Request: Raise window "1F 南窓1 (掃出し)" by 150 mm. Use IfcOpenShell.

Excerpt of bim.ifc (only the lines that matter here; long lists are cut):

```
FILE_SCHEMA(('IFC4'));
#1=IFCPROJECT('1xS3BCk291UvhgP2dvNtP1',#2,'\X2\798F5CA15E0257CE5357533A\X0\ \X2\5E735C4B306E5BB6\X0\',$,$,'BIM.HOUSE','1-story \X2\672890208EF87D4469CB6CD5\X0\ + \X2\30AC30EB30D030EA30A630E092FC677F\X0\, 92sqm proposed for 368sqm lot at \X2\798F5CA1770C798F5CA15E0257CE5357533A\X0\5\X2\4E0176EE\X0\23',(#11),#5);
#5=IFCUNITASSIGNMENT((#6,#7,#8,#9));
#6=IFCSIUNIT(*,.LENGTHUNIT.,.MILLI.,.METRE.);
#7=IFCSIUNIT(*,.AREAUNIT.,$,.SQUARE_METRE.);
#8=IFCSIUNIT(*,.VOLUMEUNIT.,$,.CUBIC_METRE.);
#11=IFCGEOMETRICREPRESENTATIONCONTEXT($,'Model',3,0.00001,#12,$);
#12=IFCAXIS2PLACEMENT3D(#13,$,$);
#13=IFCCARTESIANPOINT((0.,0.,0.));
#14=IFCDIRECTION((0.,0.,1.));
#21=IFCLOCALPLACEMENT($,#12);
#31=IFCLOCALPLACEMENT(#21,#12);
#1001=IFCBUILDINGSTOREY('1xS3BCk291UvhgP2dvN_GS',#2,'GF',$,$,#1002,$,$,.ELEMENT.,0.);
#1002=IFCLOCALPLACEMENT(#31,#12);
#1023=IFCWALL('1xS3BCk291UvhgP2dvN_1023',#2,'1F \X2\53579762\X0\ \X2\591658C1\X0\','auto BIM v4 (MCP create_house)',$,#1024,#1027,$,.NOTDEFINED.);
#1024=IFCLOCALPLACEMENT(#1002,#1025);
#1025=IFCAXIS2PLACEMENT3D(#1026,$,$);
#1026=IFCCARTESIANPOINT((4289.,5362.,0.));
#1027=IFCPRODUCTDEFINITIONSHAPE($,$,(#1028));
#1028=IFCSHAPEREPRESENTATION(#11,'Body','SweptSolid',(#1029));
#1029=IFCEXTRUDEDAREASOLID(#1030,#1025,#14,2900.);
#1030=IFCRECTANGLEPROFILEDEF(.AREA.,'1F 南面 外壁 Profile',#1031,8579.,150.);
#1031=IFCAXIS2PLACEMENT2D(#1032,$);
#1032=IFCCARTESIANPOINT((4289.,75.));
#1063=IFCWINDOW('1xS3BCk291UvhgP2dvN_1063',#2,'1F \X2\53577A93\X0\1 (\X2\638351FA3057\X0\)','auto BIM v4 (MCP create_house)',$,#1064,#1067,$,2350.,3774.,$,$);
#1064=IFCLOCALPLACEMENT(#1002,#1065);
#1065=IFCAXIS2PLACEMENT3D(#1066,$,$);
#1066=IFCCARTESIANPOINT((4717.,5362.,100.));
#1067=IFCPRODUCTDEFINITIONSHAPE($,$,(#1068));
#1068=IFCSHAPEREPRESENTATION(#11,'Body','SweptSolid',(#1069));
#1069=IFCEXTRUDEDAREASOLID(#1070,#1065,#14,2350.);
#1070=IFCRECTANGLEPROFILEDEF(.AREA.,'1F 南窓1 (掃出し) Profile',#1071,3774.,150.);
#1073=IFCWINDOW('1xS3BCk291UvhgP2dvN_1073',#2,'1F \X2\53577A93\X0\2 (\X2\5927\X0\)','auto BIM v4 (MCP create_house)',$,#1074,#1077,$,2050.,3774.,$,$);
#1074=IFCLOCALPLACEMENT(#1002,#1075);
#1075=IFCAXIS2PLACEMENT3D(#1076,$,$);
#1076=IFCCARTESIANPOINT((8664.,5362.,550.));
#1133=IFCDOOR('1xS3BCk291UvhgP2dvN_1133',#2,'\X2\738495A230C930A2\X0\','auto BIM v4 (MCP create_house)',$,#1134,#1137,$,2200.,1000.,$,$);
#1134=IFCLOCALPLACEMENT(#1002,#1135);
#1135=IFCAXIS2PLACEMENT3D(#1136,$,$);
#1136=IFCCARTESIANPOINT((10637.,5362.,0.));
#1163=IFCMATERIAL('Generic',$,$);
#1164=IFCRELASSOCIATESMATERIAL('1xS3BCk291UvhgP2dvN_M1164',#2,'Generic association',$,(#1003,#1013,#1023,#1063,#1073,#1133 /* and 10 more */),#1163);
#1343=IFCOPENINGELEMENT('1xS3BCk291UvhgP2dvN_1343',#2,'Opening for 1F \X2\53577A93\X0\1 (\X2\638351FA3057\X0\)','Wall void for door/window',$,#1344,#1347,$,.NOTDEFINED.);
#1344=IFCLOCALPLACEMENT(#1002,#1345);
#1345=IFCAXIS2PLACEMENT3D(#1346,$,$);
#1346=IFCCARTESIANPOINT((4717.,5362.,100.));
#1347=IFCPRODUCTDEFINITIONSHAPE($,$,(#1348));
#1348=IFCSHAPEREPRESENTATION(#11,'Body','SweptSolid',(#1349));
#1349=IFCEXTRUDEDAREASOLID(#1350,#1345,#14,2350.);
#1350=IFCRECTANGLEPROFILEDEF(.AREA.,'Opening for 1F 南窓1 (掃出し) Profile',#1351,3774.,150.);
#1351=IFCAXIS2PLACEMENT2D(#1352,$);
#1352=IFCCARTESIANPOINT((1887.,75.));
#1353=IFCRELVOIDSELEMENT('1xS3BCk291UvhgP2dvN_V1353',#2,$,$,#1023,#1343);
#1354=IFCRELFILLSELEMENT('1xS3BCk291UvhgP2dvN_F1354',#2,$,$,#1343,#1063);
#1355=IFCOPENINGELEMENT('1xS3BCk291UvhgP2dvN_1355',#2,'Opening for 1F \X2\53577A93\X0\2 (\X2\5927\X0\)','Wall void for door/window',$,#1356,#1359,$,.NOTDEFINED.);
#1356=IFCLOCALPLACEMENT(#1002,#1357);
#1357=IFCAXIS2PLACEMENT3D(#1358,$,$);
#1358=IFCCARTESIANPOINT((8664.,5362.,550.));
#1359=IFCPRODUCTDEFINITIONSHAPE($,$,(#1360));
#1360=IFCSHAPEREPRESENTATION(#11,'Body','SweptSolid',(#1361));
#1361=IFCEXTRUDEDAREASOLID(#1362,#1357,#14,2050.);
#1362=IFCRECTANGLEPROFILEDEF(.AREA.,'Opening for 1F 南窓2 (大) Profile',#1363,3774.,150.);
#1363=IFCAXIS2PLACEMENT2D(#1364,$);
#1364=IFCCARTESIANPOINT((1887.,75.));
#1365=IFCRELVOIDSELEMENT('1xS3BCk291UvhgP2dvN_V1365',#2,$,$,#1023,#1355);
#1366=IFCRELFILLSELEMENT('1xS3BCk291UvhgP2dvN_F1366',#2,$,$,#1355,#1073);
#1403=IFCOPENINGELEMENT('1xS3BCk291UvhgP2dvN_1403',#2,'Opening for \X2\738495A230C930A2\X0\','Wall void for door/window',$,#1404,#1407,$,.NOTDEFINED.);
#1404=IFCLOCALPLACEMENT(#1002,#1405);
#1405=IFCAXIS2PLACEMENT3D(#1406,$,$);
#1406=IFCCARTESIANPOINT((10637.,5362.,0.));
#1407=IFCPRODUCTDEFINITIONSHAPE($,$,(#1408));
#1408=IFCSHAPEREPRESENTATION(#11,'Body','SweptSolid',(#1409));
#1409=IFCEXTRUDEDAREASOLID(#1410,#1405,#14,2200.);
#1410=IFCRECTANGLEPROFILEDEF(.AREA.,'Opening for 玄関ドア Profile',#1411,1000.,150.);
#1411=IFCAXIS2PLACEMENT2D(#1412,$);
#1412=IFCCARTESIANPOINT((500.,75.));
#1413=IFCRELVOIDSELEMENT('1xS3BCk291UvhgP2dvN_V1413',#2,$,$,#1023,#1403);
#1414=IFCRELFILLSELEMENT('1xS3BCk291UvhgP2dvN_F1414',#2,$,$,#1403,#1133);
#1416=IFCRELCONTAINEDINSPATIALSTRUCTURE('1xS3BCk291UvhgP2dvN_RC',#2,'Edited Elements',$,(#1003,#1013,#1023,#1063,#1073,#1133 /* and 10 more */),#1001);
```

```python
import numpy as np
import ifcopenshell
import ifcopenshell.api.geometry
import ifcopenshell.util.placement
import ifcopenshell.util.unit

model = ifcopenshell.open("bim.ifc")
unit_scale = ifcopenshell.util.unit.calculate_unit_scale(model)

window = model.by_guid("1xS3BCk291UvhgP2dvN_1063")
opening = window.FillsVoids[0].RelatingOpeningElement
dz = 150.0

shift = np.array([0.0, 0.0, dz])
# The window is not placed relative to its opening, so move both.
for product in (opening, window):
    matrix = ifcopenshell.util.placement.get_local_placement(product.ObjectPlacement)
    matrix[:3, 3] += shift
    ifcopenshell.api.geometry.edit_object_placement(model, product=product, matrix=matrix, is_si=False)

print(f"moved by {dz * unit_scale:+.3f} m")

model.write("bim_updated.ifc")
```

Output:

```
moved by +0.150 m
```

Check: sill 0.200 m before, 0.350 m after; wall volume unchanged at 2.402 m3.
